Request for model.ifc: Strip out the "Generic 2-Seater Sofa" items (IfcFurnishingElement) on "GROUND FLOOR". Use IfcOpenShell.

First a look at what the model holds.

```python
import ifcopenshell
import ifcopenshell.util.element

model = ifcopenshell.open("model.ifc")
print(model.schema)
storey = next(s for s in model.by_type("IfcBuildingStorey") if s.Name == "GROUND FLOOR")
furniture = [e for e in ifcopenshell.util.element.get_decomposition(storey) if e.is_a("IfcFurnishingElement")]
seen = {}
for e in furniture:
    element_type = ifcopenshell.util.element.get_type(e)
    name = element_type.Name if element_type not in (None, e) else None
    seen[name] = seen.get(name, 0) + 1
for name, count in sorted(seen.items(), key=str):
    print(count, "x", name)
```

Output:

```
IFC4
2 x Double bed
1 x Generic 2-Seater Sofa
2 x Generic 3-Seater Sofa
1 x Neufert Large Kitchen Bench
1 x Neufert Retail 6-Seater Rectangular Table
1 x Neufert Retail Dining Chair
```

```python
import ifcopenshell
import ifcopenshell.api.root
import ifcopenshell.util.element

model = ifcopenshell.open("model.ifc")

storey = next(s for s in model.by_type("IfcBuildingStorey") if s.Name == "GROUND FLOOR")
furniture = [e for e in ifcopenshell.util.element.get_decomposition(storey) if e.is_a("IfcFurnishingElement")]
targets = [e for e in furniture if (t := ifcopenshell.util.element.get_type(e)) not in (None, e) and t.Name == "Generic 2-Seater Sofa"]

for e in targets:
    ifcopenshell.api.root.remove_product(model, product=e)
print(len(targets), "removed")

model.write("model_v2.ifc")
```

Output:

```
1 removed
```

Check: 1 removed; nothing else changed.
